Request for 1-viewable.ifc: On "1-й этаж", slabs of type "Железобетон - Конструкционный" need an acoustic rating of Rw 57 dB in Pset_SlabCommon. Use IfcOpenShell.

First a look at what the model holds.

```python
import ifcopenshell
import ifcopenshell.util.element

model = ifcopenshell.open("1-viewable.ifc")
print(model.schema)
storey = next(s for s in model.by_type("IfcBuildingStorey") if s.Name == "1-й этаж")
slabs = [e for e in ifcopenshell.util.element.get_decomposition(storey) if e.is_a("IfcSlab")]
seen = {}
for e in slabs:
    element_type = ifcopenshell.util.element.get_type(e)
    key = (element_type.Name if element_type != e and element_type else None, ifcopenshell.util.element.get_pset(e, "Pset_SlabCommon", "AcousticRating"))
    seen[key] = seen.get(key, 0) + 1
for (name, value), count in sorted(seen.items(), key=str):
    print(count, "x", name, "|", value)
```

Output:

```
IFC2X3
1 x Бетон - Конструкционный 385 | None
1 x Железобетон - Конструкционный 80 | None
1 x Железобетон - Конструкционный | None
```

```python
import ifcopenshell
import ifcopenshell.api.pset
import ifcopenshell.util.element

model = ifcopenshell.open("1-viewable.ifc")

storey = next(s for s in model.by_type("IfcBuildingStorey") if s.Name == "1-й этаж")
slabs = [e for e in ifcopenshell.util.element.get_decomposition(storey) if e.is_a("IfcSlab")]

count = 0
for e in slabs:
    element_type = ifcopenshell.util.element.get_type(e)
    if element_type in (None, e) or element_type.Name != "Железобетон - Конструкционный":
        continue
    # add_pset returns the element's existing set when there is one.
    pset = ifcopenshell.api.pset.add_pset(model, product=e, name="Pset_SlabCommon")
    ifcopenshell.api.pset.edit_pset(model, pset=pset, properties={"AcousticRating": "Rw 57 dB"})
    count += 1

print(count, "slabs updated")

model.write("1-viewable-out.ifc")
```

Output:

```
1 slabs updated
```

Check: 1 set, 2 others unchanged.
